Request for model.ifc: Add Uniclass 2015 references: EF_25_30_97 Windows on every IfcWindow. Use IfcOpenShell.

First a look at what the model holds.

```python
import ifcopenshell

model = ifcopenshell.open("model.ifc")
print(model.schema)
print("classifications:", [c.Name for c in model.by_type("IfcClassification")])
for ifc_class in ("IfcDoor", "IfcRoof", "IfcStair", "IfcWall", "IfcWindow"):
    print(ifc_class, len(model.by_type(ifc_class)))
```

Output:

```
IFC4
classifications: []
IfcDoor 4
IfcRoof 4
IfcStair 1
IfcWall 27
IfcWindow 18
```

```python
import ifcopenshell
import ifcopenshell.api.classification

model = ifcopenshell.open("model.ifc")

system = ifcopenshell.api.classification.add_classification(model, classification="Uniclass 2015")

codes = {
    "IfcWindow": ("EF_25_30_97", "Windows"),
}
for ifc_class, (code, name) in codes.items():
    products = model.by_type(ifc_class)
    ifcopenshell.api.classification.add_reference(
        model, products=products, classification=system, identification=code, name=name
    )
    print(code, len(products))

model.write("model-out.ifc")
```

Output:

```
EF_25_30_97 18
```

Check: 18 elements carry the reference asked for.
